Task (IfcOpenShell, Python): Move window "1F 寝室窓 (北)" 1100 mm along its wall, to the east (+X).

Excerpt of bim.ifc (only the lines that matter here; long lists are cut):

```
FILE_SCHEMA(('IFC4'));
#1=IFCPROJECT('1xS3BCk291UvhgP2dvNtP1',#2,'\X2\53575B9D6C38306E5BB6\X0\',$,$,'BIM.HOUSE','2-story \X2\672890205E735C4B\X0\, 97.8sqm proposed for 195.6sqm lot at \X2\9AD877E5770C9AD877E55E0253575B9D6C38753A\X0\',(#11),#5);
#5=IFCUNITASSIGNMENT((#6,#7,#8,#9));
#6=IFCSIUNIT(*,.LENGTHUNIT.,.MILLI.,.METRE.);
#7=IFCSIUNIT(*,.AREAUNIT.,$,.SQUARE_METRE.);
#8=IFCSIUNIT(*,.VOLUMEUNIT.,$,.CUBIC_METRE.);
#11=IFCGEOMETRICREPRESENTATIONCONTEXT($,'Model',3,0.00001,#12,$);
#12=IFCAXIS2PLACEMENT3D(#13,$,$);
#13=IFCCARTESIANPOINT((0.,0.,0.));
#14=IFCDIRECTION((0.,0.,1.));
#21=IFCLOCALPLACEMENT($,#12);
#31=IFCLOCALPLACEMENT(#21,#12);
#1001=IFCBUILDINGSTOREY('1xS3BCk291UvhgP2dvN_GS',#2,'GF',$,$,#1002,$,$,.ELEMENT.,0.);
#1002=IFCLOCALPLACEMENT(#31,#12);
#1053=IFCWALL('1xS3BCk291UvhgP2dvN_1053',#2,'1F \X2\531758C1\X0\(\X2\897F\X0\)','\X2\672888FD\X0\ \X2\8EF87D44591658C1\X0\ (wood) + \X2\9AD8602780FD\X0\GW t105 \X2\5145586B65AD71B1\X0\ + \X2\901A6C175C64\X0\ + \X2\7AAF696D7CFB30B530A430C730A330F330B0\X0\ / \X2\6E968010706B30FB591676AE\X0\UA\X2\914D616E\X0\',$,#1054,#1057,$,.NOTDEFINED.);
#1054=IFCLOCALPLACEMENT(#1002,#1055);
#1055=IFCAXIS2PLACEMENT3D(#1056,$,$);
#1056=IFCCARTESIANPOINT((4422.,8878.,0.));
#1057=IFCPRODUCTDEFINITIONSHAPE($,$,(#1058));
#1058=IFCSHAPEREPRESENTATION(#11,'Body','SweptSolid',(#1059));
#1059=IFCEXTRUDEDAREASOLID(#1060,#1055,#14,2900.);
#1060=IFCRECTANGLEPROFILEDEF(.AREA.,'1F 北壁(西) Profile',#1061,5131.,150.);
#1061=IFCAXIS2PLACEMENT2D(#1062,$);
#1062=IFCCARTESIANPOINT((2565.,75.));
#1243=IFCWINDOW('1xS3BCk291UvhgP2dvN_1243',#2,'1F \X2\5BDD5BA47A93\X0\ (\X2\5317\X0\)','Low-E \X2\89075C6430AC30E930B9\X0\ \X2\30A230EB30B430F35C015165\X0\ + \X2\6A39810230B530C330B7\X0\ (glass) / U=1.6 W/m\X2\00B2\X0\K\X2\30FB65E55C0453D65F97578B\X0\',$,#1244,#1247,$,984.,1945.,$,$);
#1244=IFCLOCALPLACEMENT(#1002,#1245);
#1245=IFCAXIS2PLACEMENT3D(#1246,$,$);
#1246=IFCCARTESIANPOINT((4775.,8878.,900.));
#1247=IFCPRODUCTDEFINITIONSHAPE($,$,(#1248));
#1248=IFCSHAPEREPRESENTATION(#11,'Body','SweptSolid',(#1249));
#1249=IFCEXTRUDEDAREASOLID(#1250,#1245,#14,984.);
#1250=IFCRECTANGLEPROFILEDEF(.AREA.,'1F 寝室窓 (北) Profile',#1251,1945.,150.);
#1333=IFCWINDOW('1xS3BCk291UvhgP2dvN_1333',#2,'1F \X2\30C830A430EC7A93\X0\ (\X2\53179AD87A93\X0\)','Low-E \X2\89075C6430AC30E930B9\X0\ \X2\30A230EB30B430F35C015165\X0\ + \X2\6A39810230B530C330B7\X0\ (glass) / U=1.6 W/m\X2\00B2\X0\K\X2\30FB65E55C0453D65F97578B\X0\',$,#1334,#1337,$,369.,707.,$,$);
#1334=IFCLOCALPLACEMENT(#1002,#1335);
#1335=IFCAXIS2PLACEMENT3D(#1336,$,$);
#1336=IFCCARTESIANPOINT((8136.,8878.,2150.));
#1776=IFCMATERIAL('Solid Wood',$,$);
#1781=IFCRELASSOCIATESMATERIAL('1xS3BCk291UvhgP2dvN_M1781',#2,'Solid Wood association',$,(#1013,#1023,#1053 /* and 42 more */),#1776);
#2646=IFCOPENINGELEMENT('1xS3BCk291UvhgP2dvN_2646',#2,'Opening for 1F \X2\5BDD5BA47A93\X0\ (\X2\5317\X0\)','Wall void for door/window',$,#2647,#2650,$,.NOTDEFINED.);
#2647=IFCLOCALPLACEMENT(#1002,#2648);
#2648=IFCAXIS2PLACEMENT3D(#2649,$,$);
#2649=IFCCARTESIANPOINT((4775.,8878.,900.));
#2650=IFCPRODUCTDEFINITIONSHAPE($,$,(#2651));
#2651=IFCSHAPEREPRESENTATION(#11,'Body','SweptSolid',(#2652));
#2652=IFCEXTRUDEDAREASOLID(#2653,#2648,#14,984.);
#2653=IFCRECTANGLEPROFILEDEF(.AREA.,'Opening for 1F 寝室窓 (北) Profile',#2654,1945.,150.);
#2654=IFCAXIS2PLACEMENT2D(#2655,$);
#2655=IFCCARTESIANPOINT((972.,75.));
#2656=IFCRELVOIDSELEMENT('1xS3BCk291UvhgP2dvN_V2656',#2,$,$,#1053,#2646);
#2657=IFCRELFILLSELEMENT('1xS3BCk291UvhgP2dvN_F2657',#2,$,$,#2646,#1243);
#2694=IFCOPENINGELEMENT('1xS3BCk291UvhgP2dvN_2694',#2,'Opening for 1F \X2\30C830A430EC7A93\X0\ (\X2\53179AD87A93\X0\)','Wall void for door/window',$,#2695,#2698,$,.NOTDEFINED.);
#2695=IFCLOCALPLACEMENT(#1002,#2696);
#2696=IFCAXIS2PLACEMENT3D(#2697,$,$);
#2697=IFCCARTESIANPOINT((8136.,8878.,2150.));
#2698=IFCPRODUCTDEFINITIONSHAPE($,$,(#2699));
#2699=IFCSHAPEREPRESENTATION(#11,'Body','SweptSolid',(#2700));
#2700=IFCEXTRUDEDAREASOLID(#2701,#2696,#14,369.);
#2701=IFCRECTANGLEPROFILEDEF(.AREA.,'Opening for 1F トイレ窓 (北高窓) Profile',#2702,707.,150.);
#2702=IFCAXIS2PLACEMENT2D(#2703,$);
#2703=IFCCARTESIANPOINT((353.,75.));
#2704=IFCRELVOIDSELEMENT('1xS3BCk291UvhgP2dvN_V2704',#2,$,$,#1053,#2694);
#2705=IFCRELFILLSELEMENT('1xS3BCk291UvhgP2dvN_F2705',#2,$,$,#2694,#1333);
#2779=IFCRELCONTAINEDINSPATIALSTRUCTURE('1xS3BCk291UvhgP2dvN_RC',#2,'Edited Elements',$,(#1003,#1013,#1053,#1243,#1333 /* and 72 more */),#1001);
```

```python
import ifcopenshell
import ifcopenshell.api.geometry
import ifcopenshell.util.placement
import ifcopenshell.util.unit

model = ifcopenshell.open("bim.ifc")
unit_scale = ifcopenshell.util.unit.calculate_unit_scale(model)

window = model.by_guid("1xS3BCk291UvhgP2dvN_1243")
opening = window.FillsVoids[0].RelatingOpeningElement
wall = opening.VoidsElements[0].RelatingBuildingElement

wall_matrix = ifcopenshell.util.placement.get_local_placement(wall.ObjectPlacement)
shift = wall_matrix[:3, 0] * 1.1 / unit_scale
before = ifcopenshell.util.placement.get_local_placement(window.ObjectPlacement)[:3, 3].copy()

# The window is not placed relative to its opening, so move both.
for product in (opening, window):
    matrix = ifcopenshell.util.placement.get_local_placement(product.ObjectPlacement)
    matrix[:3, 3] += shift
    ifcopenshell.api.geometry.edit_object_placement(model, product=product, matrix=matrix, is_si=False)

after = ifcopenshell.util.placement.get_local_placement(window.ObjectPlacement)[:3, 3]
print("window moved by", (after - before).round(3) + 0.0)

model.write("bim_rev.ifc")
```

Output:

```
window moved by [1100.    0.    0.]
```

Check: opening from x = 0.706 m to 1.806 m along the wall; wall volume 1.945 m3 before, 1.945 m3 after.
